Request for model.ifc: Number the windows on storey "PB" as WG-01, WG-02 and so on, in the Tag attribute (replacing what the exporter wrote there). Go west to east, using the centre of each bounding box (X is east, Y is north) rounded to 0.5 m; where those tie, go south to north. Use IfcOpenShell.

First a look at what the model holds.

```python
import ifcopenshell
import ifcopenshell.util.element
import ifcopenshell.util.placement

model = ifcopenshell.open("model.ifc")
print(model.schema)
storey = next(s for s in model.by_type("IfcBuildingStorey") if s.Name == "PB")
windows = [e for e in ifcopenshell.util.element.get_decomposition(storey) if e.is_a("IfcWindow")]
for e in sorted(windows, key=lambda e: e.id()):
    origin = ifcopenshell.util.placement.get_local_placement(e.ObjectPlacement)[:3, 3]
    print(e.id(), e.Tag, e.Name, origin.round(2) + 0.0, sep=" | ")
```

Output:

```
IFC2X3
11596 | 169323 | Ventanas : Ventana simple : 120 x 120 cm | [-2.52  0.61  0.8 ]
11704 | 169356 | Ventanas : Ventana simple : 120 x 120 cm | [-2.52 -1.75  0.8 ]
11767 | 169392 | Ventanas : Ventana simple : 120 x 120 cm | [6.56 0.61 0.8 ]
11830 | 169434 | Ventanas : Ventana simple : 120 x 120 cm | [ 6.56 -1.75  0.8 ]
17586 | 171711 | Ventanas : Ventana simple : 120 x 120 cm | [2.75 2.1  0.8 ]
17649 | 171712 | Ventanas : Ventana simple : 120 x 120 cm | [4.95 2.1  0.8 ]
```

```python
import ifcopenshell
import ifcopenshell.geom
import ifcopenshell.util.element
import ifcopenshell.util.shape

model = ifcopenshell.open("model.ifc")
settings = ifcopenshell.geom.settings()
settings.set("use-world-coords", True)


def centre(element):
    shape = ifcopenshell.geom.create_shape(settings, element)
    return ifcopenshell.util.shape.get_bbox_centroid(shape.geometry)


storey = next(s for s in model.by_type("IfcBuildingStorey") if s.Name == "PB")
windows = [e for e in ifcopenshell.util.element.get_decomposition(storey) if e.is_a("IfcWindow")]

# Insertion points can sit at a corner or the storey origin, so sort by the geometry (in metres).
centres = {e: centre(e) for e in windows}
windows.sort(key=lambda e: (round(centres[e][0] / 0.5), centres[e][1]))

for i, e in enumerate(windows, start=1):
    number = f"WG-{i:02d}"
    e.Tag = number
    print(e.id(), number)

model.write("model_edited.ifc")
```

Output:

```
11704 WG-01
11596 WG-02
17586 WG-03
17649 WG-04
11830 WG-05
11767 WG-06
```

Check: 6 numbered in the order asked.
